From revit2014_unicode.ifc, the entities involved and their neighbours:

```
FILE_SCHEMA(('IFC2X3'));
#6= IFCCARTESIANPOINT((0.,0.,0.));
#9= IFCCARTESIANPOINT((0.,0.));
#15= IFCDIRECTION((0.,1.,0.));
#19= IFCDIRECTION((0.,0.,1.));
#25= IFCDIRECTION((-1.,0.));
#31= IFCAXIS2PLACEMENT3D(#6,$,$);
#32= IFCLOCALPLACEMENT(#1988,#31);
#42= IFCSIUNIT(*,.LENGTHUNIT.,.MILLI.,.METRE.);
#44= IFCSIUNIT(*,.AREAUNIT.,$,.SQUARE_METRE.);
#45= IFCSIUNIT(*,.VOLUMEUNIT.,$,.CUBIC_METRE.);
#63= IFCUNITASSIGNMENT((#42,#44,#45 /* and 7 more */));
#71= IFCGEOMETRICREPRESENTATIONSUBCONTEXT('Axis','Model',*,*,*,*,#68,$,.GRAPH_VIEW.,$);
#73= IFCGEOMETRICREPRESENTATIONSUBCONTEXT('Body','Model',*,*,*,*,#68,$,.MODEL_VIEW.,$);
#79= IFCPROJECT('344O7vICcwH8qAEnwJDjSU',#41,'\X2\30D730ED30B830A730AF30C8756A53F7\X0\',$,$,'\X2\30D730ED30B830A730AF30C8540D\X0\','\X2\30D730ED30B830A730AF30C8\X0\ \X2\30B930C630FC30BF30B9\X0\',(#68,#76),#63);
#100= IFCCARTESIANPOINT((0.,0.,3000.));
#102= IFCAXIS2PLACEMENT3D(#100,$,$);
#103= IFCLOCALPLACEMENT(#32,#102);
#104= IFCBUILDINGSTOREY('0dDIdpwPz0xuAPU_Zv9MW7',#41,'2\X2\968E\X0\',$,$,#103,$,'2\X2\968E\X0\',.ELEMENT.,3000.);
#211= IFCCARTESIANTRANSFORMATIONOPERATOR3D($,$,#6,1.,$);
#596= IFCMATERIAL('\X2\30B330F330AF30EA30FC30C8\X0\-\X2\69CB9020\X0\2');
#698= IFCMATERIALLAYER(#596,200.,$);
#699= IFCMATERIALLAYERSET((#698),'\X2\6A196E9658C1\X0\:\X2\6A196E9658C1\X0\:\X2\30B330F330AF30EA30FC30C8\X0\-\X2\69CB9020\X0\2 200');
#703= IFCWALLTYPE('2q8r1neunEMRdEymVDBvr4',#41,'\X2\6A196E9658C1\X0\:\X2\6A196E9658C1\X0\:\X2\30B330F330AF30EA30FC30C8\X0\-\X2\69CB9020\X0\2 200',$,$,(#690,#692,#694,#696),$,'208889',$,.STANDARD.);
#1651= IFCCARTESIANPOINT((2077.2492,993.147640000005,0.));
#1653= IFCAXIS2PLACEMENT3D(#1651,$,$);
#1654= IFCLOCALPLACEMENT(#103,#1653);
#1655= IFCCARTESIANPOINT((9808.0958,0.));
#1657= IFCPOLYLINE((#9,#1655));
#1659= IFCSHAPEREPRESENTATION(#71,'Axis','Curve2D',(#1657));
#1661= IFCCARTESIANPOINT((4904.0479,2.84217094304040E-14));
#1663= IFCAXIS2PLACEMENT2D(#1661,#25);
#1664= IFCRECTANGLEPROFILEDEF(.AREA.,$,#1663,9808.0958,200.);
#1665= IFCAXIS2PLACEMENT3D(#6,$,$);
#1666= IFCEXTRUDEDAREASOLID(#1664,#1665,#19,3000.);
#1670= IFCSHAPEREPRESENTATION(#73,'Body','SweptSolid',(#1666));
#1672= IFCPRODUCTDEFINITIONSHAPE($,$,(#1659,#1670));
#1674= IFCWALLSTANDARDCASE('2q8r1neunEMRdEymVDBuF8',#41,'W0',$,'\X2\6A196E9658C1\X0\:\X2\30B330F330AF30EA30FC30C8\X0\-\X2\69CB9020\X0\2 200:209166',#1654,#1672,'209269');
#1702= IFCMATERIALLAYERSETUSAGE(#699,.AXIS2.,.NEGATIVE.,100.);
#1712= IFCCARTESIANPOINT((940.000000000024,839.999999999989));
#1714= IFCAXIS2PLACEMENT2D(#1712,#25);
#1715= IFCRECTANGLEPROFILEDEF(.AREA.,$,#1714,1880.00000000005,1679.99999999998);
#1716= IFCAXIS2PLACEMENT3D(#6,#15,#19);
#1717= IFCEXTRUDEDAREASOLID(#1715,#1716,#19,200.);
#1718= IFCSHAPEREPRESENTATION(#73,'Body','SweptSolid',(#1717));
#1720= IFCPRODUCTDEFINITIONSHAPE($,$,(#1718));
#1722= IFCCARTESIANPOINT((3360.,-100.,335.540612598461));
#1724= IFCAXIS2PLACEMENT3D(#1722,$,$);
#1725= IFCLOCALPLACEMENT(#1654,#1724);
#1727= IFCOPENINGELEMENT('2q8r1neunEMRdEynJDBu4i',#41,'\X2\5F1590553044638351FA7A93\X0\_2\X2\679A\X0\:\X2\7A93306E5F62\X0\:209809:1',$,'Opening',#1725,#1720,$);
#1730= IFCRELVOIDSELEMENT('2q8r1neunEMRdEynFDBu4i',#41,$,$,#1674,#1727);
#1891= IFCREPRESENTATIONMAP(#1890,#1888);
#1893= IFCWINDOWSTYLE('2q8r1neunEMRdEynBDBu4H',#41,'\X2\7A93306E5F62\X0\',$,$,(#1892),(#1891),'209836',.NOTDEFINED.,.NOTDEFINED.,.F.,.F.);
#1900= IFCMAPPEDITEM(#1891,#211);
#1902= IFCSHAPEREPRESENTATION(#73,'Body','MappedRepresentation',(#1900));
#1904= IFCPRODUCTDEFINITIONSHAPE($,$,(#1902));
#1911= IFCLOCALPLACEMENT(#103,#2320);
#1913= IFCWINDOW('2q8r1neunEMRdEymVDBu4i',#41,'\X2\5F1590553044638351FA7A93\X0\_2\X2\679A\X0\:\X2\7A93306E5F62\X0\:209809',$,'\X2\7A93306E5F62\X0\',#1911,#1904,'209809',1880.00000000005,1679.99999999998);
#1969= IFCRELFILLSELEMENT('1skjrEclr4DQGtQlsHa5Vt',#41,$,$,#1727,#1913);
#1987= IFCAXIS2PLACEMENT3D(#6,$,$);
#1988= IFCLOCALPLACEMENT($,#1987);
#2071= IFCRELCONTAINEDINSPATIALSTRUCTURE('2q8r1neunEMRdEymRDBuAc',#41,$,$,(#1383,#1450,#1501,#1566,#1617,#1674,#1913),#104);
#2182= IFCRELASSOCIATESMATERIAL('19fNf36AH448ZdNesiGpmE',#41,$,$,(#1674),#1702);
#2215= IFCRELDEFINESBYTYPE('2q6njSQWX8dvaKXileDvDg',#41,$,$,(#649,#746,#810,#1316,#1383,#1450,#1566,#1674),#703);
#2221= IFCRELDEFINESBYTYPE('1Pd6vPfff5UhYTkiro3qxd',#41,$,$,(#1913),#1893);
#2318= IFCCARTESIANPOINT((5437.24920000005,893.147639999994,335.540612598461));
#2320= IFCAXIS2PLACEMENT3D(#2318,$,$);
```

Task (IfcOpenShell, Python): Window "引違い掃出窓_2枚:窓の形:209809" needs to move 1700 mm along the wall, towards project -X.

```python
import ifcopenshell
import ifcopenshell.api.geometry
import ifcopenshell.util.placement
import ifcopenshell.util.unit

model = ifcopenshell.open("revit2014_unicode.ifc")
unit_scale = ifcopenshell.util.unit.calculate_unit_scale(model)

window = model.by_guid("2q8r1neunEMRdEymVDBu4i")
opening = window.FillsVoids[0].RelatingOpeningElement
wall = opening.VoidsElements[0].RelatingBuildingElement

wall_matrix = ifcopenshell.util.placement.get_local_placement(wall.ObjectPlacement)
shift = wall_matrix[:3, 0] * -1.7 / unit_scale
before = ifcopenshell.util.placement.get_local_placement(window.ObjectPlacement)[:3, 3].copy()

# The window is not placed relative to its opening, so move both.
for product in (opening, window):
    matrix = ifcopenshell.util.placement.get_local_placement(product.ObjectPlacement)
    matrix[:3, 3] += shift
    ifcopenshell.api.geometry.edit_object_placement(model, product=product, matrix=matrix, is_si=False)

after = ifcopenshell.util.placement.get_local_placement(window.ObjectPlacement)[:3, 3]
print("window moved by", (after - before).round(3) + 0.0)

model.write("revit2014_unicode_updated.ifc")
```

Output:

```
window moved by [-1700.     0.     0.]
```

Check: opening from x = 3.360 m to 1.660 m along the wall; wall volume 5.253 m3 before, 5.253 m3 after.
